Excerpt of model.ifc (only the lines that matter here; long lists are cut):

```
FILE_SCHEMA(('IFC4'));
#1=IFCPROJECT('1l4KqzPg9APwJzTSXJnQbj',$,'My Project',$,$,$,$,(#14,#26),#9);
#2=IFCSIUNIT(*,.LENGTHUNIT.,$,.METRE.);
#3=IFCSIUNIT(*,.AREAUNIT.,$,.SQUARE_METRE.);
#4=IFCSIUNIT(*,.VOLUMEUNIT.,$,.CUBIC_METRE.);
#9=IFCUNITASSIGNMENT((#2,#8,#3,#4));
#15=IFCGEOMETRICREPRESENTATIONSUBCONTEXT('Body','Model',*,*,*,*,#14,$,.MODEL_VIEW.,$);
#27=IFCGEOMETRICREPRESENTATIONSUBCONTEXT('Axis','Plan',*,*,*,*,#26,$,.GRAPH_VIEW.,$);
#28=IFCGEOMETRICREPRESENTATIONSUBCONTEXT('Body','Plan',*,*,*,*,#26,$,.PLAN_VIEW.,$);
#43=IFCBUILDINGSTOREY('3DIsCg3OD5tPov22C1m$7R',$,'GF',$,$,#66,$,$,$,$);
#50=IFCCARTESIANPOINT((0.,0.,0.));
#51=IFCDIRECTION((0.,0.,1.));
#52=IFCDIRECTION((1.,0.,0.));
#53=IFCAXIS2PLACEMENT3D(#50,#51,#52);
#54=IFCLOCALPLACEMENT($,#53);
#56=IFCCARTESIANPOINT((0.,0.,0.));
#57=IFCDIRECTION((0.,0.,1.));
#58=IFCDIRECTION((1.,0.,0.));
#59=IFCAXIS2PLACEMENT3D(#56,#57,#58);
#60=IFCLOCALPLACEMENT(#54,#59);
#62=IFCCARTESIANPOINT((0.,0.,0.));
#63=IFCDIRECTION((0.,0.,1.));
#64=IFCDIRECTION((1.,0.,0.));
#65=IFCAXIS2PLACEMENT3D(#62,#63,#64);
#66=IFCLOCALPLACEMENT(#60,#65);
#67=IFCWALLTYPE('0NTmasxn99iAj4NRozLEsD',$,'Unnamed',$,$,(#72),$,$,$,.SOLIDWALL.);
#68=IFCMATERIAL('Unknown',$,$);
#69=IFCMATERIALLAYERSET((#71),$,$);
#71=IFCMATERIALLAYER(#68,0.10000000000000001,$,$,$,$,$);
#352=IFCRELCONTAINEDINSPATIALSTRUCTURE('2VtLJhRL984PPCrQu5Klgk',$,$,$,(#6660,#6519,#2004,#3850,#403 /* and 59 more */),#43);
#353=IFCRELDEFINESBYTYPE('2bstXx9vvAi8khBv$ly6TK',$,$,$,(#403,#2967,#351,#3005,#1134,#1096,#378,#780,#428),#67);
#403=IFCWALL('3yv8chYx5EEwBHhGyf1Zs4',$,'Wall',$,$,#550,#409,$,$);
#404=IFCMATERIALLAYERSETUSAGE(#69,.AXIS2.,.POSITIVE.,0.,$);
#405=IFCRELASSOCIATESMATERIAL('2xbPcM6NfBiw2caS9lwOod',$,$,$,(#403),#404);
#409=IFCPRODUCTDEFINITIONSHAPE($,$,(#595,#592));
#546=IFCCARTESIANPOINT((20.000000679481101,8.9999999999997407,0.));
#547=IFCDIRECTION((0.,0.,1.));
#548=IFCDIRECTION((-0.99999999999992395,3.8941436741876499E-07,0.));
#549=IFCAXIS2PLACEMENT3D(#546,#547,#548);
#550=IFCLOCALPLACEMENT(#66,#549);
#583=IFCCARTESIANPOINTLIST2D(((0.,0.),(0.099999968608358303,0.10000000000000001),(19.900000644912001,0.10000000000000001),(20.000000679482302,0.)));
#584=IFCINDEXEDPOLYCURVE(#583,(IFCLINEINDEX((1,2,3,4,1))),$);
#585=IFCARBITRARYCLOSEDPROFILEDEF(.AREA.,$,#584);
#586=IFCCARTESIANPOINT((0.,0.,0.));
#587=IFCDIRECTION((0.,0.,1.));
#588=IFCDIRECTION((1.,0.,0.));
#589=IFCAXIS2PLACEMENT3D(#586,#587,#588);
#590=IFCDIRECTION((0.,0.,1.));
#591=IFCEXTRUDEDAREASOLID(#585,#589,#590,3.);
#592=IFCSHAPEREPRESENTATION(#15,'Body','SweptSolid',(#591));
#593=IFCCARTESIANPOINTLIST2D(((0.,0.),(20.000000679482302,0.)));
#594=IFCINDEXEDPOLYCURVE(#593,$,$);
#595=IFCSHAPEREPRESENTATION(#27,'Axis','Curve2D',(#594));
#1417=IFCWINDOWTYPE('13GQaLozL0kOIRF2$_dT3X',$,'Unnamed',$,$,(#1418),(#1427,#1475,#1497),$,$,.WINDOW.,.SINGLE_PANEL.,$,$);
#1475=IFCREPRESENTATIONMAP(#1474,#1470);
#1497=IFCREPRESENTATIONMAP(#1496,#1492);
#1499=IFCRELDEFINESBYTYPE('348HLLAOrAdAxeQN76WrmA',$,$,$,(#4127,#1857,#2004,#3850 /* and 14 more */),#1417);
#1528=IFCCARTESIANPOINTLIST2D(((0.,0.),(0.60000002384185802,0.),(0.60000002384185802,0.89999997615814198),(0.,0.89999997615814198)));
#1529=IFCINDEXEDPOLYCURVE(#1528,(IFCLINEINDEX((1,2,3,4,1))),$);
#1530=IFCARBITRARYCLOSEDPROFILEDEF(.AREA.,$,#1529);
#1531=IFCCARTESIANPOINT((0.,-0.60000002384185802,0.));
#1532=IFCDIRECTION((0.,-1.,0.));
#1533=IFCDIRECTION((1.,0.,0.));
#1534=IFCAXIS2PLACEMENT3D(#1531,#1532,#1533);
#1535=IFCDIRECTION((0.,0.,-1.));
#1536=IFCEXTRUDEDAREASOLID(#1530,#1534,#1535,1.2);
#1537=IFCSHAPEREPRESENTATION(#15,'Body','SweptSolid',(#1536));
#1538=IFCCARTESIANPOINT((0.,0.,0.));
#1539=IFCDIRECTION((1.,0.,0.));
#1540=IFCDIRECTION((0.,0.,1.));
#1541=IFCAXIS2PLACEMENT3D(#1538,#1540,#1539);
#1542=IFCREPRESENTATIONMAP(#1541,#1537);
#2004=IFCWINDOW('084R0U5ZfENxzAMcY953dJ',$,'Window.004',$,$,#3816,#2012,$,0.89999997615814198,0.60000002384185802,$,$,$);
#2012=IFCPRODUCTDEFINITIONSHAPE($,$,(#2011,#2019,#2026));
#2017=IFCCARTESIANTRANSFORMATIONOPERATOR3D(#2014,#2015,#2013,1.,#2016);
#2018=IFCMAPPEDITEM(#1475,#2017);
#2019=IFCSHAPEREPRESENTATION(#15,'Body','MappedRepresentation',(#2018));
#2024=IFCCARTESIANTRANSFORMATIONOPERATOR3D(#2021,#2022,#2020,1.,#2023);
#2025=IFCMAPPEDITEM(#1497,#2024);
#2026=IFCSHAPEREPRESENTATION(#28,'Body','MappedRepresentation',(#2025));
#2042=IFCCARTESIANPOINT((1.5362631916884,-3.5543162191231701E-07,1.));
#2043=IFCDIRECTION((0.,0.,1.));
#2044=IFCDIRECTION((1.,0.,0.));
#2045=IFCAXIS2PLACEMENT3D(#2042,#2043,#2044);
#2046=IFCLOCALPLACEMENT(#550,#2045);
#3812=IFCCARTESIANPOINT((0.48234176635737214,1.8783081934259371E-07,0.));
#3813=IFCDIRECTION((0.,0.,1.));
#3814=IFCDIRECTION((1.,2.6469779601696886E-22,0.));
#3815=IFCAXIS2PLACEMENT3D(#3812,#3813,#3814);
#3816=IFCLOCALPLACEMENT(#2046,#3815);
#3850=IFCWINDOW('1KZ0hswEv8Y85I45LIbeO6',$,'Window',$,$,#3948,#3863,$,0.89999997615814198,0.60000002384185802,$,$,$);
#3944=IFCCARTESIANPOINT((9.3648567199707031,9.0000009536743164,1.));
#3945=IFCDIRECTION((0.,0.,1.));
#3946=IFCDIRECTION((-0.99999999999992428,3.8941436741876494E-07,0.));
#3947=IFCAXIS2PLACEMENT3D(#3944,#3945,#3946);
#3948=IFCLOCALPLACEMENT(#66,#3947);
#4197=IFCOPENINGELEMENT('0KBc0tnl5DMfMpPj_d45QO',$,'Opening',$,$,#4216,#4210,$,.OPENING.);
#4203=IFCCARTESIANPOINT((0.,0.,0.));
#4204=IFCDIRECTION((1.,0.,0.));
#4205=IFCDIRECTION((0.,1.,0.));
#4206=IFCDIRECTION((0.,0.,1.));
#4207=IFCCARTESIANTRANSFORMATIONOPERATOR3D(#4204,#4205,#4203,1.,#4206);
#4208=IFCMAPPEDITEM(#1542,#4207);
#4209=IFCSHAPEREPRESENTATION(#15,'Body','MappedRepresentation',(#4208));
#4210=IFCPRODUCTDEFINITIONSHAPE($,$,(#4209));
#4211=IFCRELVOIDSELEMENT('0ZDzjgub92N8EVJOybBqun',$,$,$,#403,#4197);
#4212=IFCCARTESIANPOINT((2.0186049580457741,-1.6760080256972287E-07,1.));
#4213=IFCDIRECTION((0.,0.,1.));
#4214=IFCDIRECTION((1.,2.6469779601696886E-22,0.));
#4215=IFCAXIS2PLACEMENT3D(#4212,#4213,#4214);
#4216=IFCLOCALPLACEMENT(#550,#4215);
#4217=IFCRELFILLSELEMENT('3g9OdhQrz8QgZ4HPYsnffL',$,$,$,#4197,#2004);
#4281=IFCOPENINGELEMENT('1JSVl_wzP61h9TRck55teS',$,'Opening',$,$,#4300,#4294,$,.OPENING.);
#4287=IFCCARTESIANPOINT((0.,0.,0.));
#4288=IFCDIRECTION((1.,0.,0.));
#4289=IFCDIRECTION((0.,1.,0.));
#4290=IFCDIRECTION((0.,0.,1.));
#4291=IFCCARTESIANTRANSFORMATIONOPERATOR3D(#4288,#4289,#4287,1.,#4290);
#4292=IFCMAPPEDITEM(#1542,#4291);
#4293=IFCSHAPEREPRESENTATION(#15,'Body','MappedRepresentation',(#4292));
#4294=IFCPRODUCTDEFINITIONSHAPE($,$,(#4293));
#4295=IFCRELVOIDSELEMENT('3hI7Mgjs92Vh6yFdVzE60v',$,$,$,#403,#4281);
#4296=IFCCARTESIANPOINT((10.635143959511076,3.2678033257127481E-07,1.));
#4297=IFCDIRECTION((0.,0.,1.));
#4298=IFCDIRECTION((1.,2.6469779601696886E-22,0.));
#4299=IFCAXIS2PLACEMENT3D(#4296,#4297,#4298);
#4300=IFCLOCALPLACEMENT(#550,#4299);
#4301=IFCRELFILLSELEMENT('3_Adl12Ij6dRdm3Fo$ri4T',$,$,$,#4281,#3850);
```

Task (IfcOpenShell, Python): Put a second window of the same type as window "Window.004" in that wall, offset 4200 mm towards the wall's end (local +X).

```python
import ifcopenshell
import ifcopenshell.api.feature
import ifcopenshell.api.geometry
import ifcopenshell.api.root
import ifcopenshell.geom
import ifcopenshell.util.element
import ifcopenshell.util.placement
import ifcopenshell.util.shape
import ifcopenshell.util.unit

model = ifcopenshell.open("model.ifc")
unit_scale = ifcopenshell.util.unit.calculate_unit_scale(model)
settings = ifcopenshell.geom.settings()


def volume(element):
    """Net volume in cubic metres, openings subtracted."""
    shape = ifcopenshell.geom.create_shape(settings, element)
    return ifcopenshell.util.shape.get_volume(shape.geometry)


window = model.by_id(2004)
opening = window.FillsVoids[0].RelatingOpeningElement
wall = opening.VoidsElements[0].RelatingBuildingElement
before = volume(wall)
shift = ifcopenshell.util.placement.get_local_placement(wall.ObjectPlacement)[:3, 0] * 4.2 / unit_scale

# copy_class copies the void relationship, type, container and properties, but no geometry.
new_opening = ifcopenshell.api.root.copy_class(model, product=opening)
new_opening.Representation = ifcopenshell.util.element.copy_deep(
    model, opening.Representation, exclude=["IfcGeometricRepresentationContext", "IfcRepresentationMap"]
)
new_window = ifcopenshell.api.root.copy_class(model, product=window)
new_window.Representation = ifcopenshell.util.element.copy_deep(
    model, window.Representation, exclude=["IfcGeometricRepresentationContext", "IfcRepresentationMap"]
)
ifcopenshell.api.feature.add_filling(model, opening=new_opening, element=new_window)

for old, new in ((opening, new_opening), (window, new_window)):
    matrix = ifcopenshell.util.placement.get_local_placement(old.ObjectPlacement)
    matrix[:3, 3] += shift
    ifcopenshell.api.geometry.edit_object_placement(model, product=new, matrix=matrix, is_si=False)

after = volume(wall)

print(f"wall volume {before:.3f} -> {after:.3f} m3")

model.write("model_edited.ifc")
```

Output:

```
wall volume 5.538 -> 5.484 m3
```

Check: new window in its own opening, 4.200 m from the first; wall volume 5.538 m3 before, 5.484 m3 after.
